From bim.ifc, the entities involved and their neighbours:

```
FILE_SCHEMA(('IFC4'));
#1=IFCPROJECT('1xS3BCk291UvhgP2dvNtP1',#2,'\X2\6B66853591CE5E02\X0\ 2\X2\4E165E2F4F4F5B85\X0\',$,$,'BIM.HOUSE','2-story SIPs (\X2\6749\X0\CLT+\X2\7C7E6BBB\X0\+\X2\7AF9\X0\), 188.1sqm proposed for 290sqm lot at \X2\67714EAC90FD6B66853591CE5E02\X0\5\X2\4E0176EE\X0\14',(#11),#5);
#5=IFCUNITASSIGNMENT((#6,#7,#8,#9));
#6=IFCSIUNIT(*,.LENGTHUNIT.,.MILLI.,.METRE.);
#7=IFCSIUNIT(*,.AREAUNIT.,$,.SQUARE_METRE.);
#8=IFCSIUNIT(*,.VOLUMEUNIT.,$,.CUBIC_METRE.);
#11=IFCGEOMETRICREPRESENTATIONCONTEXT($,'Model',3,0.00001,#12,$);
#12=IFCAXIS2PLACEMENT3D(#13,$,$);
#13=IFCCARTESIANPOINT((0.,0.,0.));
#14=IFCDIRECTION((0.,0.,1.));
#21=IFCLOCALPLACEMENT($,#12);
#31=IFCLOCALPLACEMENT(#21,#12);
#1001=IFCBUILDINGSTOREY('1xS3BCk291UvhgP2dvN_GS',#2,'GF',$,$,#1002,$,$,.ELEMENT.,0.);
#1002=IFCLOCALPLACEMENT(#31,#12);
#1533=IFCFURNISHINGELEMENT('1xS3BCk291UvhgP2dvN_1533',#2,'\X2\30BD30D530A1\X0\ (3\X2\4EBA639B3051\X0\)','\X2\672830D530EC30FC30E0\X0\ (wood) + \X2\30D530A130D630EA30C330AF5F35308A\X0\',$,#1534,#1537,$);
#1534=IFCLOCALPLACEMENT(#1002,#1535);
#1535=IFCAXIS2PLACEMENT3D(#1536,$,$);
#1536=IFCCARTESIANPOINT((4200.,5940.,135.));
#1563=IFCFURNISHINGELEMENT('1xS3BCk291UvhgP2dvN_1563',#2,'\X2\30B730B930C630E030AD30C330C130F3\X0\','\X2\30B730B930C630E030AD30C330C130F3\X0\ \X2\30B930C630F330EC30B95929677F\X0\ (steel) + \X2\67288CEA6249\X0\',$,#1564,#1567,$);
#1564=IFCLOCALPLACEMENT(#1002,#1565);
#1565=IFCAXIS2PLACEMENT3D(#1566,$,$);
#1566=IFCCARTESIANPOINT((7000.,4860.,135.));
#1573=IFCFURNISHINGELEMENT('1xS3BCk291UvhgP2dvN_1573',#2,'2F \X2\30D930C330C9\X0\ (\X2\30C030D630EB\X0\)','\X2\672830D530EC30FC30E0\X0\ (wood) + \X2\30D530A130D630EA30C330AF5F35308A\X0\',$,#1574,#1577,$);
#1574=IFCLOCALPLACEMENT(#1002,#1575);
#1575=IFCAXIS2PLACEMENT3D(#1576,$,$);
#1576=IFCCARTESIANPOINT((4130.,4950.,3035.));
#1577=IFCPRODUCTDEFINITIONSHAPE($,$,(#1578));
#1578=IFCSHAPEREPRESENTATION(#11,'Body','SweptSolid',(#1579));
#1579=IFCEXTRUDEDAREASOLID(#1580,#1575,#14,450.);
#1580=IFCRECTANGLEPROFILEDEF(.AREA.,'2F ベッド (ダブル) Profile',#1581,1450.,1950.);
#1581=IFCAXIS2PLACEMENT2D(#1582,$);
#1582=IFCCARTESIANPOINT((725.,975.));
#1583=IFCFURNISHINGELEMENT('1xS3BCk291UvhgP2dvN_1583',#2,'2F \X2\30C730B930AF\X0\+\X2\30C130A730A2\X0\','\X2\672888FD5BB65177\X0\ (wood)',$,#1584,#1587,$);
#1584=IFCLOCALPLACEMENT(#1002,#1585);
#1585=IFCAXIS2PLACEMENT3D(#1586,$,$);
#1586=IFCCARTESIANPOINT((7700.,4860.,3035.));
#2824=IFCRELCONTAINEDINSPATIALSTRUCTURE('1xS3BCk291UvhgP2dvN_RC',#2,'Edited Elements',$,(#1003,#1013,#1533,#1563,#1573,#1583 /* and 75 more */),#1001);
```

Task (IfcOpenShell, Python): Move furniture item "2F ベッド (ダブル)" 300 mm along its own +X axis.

```python
import ifcopenshell
import ifcopenshell.api.geometry
import ifcopenshell.util.placement

model = ifcopenshell.open("bim.ifc")

item = model.by_guid("1xS3BCk291UvhgP2dvN_1573")
matrix = ifcopenshell.util.placement.get_local_placement(item.ObjectPlacement)
matrix[:3, 3] += matrix[:3, 0] * 300.0
ifcopenshell.api.geometry.edit_object_placement(model, product=item, matrix=matrix, is_si=False)

print(ifcopenshell.util.placement.get_local_placement(item.ObjectPlacement).round(3) + 0.0)

model.write("bim_updated.ifc")
```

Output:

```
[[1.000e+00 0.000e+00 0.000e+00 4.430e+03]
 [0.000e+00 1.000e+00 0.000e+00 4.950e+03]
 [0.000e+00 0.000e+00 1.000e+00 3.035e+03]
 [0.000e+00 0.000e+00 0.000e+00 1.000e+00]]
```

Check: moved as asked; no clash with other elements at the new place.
